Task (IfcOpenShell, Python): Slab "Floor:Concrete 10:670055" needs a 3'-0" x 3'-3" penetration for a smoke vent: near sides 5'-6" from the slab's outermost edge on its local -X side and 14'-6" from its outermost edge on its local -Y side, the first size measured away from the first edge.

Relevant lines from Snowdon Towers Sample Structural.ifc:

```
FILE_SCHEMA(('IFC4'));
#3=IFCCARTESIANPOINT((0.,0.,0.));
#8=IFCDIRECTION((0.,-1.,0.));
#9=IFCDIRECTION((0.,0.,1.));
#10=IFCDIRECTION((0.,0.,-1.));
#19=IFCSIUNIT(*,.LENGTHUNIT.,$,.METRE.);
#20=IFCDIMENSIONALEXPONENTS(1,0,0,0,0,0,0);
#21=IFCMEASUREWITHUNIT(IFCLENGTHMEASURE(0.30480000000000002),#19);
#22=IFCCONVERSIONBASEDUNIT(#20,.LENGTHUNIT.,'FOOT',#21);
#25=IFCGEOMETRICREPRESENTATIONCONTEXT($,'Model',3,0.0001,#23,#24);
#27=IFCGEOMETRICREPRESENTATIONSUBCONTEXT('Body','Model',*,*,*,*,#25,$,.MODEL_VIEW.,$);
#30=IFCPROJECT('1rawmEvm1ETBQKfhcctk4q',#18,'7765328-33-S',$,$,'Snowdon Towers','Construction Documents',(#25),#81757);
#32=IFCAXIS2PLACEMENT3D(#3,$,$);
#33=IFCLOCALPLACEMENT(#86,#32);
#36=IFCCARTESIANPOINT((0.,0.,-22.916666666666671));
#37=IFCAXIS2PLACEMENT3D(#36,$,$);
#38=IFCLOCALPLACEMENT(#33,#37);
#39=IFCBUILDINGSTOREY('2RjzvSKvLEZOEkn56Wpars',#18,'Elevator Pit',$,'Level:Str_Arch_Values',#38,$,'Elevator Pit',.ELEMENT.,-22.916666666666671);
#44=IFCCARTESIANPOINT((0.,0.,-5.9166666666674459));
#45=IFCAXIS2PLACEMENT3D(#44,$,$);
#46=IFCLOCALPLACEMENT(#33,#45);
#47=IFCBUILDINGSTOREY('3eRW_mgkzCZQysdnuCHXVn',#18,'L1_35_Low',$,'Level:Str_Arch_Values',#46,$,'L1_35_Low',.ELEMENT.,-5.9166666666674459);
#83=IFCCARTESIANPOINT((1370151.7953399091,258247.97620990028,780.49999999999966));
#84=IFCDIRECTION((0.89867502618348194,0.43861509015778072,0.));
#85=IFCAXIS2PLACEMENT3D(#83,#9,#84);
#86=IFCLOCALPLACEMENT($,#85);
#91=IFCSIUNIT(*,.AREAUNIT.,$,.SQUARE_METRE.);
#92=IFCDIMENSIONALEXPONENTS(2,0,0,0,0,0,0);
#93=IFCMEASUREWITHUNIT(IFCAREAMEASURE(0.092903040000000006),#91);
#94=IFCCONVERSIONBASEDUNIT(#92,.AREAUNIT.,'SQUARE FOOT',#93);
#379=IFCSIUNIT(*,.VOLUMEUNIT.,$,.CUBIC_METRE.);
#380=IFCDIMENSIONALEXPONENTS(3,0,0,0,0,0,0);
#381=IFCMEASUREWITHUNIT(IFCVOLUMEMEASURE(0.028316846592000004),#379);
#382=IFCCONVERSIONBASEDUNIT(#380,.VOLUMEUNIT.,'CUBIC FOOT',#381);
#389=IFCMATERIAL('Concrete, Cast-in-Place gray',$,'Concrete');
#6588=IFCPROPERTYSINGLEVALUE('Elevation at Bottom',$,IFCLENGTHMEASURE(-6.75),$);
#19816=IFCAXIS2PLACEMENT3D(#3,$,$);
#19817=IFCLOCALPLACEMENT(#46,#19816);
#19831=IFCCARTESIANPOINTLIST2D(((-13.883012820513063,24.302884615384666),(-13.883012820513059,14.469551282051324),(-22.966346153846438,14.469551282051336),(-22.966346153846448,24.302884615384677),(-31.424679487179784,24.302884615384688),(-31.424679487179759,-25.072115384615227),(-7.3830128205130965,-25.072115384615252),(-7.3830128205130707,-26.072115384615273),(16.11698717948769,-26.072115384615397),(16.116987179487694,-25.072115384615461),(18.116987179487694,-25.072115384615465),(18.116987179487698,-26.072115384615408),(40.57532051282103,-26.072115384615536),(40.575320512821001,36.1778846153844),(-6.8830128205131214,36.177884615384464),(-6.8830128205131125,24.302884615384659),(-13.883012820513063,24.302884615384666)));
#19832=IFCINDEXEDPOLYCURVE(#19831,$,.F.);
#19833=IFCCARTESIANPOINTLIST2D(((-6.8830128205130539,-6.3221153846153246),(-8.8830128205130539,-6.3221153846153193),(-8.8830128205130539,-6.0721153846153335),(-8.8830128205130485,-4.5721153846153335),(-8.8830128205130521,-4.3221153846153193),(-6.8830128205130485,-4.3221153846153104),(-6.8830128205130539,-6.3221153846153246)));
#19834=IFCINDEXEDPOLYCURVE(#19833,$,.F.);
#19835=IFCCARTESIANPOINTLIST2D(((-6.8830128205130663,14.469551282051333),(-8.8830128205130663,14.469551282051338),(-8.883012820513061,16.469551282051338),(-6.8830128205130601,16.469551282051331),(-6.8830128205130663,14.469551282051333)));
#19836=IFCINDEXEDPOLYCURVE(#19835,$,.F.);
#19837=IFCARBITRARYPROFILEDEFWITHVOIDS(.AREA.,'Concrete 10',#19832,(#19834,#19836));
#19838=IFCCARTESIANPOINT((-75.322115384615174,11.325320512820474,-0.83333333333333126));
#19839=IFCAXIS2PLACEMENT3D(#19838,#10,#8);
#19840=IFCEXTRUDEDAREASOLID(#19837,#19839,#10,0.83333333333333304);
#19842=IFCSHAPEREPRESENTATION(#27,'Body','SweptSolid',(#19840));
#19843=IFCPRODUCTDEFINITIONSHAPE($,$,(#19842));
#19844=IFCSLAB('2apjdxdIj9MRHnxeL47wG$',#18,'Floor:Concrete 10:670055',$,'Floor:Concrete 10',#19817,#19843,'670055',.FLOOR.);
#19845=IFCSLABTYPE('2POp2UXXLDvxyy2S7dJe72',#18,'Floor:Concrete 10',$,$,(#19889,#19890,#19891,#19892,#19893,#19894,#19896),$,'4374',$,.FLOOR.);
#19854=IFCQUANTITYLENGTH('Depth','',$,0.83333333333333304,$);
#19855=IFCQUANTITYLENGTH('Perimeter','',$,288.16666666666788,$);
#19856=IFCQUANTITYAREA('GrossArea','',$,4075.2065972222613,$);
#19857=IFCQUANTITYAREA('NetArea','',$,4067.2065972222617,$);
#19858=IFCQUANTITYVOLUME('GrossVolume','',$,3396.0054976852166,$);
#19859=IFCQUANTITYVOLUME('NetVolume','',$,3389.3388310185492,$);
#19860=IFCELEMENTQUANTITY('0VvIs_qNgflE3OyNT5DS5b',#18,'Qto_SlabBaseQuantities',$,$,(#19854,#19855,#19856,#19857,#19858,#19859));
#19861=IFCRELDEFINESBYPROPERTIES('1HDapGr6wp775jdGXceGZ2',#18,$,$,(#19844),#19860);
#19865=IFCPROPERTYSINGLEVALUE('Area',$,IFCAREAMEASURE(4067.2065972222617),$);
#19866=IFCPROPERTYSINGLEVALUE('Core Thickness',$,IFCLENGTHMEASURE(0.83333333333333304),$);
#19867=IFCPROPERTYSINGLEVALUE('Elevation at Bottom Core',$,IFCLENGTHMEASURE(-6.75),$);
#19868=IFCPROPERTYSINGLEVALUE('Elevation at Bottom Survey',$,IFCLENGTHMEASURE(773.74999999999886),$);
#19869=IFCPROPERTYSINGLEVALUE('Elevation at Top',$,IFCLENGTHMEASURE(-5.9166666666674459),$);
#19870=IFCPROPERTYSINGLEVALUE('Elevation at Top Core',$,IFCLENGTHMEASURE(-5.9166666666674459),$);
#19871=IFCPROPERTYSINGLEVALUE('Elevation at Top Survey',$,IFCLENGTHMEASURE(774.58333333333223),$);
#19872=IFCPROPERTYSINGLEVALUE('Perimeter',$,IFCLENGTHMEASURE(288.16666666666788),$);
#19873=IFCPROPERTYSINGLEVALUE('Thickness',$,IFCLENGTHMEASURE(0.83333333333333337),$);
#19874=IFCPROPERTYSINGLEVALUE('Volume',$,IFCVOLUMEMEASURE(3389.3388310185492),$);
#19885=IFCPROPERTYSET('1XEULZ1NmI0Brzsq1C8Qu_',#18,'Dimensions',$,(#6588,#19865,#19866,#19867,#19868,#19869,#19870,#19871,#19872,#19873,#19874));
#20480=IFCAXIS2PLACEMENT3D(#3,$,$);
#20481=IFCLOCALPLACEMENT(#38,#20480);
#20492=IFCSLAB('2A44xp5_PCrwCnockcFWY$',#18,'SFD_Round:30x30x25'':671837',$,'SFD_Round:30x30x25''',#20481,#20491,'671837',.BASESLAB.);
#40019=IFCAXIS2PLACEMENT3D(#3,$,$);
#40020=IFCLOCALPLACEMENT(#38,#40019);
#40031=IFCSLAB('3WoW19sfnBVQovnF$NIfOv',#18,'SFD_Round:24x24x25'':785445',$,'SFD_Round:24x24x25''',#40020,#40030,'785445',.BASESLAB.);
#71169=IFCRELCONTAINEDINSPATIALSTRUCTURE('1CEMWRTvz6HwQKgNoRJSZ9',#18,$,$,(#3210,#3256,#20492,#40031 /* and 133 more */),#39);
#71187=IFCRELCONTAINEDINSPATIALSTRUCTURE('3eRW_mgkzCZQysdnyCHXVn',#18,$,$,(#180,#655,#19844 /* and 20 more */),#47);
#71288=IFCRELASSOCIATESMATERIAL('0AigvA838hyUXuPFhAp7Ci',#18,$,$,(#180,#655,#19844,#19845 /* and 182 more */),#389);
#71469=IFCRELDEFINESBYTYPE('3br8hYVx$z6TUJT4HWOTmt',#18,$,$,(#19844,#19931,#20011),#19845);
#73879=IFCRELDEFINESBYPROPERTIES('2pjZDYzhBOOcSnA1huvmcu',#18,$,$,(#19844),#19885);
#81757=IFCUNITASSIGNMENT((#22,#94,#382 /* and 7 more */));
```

```python
import numpy as np
import ifcopenshell
import ifcopenshell.api.feature
import ifcopenshell.api.geometry
import ifcopenshell.api.pset
import ifcopenshell.api.root
import ifcopenshell.geom
import ifcopenshell.util.element
import ifcopenshell.util.placement
import ifcopenshell.util.representation
import ifcopenshell.util.shape
import ifcopenshell.util.unit

model = ifcopenshell.open("Snowdon Towers Sample Structural.ifc")
unit_scale = ifcopenshell.util.unit.calculate_unit_scale(model)
area_scale = ifcopenshell.util.unit.calculate_unit_scale(model, "AREAUNIT")
volume_scale = ifcopenshell.util.unit.calculate_unit_scale(model, "VOLUMEUNIT")
settings = ifcopenshell.geom.settings()


def volume(element):
    """Net volume in cubic metres, openings subtracted."""
    shape = ifcopenshell.geom.create_shape(settings, element)
    return ifcopenshell.util.shape.get_volume(shape.geometry)


slab = model.by_guid("2apjdxdIj9MRHnxeL47wG$")
before = volume(slab)

# Extent in the slab's own axes, in metres. The edges named are its -X and -Y sides.
slab_shape = ifcopenshell.geom.create_shape(settings, slab)
vertices = ifcopenshell.util.shape.get_vertices(slab_shape.geometry)
x_min, y_min, bottom = vertices.min(axis=0)
top = vertices[:, 2].max()

opening = ifcopenshell.api.root.create_entity(model, ifc_class="IfcOpeningElement", name="Smoke vent opening", predefined_type="OPENING")
context = ifcopenshell.util.representation.get_context(model, "Model", "Body", "MODEL_VIEW")
width, depth = 0.9144, 0.9906
outline = [(0.0, 0.0), (width, 0.0), (width, depth), (0.0, depth), (0.0, 0.0)]
# Overshoot both faces by 50 mm so the cut is clean.
shape = ifcopenshell.api.geometry.add_slab_representation(
    model, context=context, depth=top - bottom + 0.1, polyline=outline
)
ifcopenshell.api.geometry.assign_representation(model, product=opening, representation=shape)

matrix = ifcopenshell.util.placement.get_local_placement(slab.ObjectPlacement)
matrix[:, 3] = matrix @ np.append(np.array([x_min + 1.6764, y_min + 4.4196, bottom - 0.05]) / unit_scale, 1.0)
ifcopenshell.api.geometry.edit_object_placement(model, product=opening, matrix=matrix, is_si=False)
ifcopenshell.api.feature.add_feature(model, feature=opening, element=slab)

after = volume(slab)

# Update the slab's stored quantities.
qto = model.by_id(ifcopenshell.util.element.get_pset(slab, "Qto_SlabBaseQuantities", should_inherit=False)["id"])
ifcopenshell.api.pset.edit_qto(model, qto=qto, properties={
    "NetArea": after / (top - bottom) / area_scale,
    "NetVolume": after / volume_scale,
})
pset = model.by_id(ifcopenshell.util.element.get_pset(slab, "Dimensions", should_inherit=False)["id"])
ifcopenshell.api.pset.edit_pset(model, pset=pset, properties={
    "Area": model.create_entity("IfcAreaMeasure", after / (top - bottom) / area_scale),
    "Volume": model.create_entity("IfcVolumeMeasure", after / volume_scale),
})

print(f"slab volume {before:.3f} -> {after:.3f} m3")

model.write("Snowdon Towers Sample Structural_edited.ifc")
```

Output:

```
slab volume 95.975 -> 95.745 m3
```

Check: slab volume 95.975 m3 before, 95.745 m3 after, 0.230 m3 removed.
